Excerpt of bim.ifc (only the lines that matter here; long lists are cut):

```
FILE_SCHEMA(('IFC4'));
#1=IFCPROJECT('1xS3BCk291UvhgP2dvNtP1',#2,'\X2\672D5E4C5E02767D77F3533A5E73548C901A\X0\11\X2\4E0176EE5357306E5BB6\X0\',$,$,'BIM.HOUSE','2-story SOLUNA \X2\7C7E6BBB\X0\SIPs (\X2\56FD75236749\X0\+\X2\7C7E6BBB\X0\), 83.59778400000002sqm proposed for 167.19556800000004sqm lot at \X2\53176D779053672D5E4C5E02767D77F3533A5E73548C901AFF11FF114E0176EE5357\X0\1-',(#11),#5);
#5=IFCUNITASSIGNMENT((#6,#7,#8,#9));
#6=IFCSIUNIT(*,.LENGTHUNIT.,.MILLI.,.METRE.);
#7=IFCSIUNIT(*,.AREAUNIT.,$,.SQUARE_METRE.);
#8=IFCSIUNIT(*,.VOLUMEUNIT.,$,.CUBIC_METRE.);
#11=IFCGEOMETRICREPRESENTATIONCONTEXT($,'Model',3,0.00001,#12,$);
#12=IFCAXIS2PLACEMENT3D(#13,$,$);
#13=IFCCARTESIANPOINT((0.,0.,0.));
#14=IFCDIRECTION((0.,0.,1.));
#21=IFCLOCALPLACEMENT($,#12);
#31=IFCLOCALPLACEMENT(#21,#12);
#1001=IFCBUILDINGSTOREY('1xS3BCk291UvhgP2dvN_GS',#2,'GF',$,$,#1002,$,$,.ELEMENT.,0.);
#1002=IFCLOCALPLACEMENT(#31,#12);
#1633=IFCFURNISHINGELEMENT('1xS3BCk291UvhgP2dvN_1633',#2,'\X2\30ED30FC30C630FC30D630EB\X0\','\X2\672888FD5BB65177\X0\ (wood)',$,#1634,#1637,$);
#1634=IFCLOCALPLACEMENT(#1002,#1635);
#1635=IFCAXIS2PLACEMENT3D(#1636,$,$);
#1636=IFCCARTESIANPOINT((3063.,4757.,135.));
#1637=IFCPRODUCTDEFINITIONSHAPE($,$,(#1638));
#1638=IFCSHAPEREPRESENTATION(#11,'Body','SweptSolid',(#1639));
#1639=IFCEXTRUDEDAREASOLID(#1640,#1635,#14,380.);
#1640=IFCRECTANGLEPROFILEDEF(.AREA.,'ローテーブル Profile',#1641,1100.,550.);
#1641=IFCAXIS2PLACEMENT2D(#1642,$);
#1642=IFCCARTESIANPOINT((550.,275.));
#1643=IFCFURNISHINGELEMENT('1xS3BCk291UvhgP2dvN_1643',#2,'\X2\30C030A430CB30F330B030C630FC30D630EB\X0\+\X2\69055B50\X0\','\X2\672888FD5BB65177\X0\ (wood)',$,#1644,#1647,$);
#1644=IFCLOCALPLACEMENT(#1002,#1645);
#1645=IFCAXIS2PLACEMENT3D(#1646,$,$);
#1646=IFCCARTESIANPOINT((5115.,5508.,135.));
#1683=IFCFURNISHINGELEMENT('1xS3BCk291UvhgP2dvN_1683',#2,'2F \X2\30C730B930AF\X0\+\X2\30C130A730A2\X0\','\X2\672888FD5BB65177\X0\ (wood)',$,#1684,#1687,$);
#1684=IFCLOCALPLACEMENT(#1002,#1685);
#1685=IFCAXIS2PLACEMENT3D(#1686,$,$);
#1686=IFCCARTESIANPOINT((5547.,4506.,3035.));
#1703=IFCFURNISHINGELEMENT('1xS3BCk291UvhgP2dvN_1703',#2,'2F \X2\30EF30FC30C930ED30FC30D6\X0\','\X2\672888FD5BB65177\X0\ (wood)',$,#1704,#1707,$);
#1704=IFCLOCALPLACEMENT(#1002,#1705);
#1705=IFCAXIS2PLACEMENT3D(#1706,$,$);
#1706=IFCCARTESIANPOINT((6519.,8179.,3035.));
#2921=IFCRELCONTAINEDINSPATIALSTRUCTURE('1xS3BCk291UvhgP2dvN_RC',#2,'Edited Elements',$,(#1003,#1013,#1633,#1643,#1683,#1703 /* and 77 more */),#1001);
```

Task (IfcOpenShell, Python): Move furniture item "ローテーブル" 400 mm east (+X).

```python
import ifcopenshell
import ifcopenshell.api.geometry
import ifcopenshell.util.placement
import ifcopenshell.util.unit

model = ifcopenshell.open("bim.ifc")
unit_scale = ifcopenshell.util.unit.calculate_unit_scale(model)

item = model.by_guid("1xS3BCk291UvhgP2dvN_1633")
matrix = ifcopenshell.util.placement.get_local_placement(item.ObjectPlacement)
matrix[0, 3] += 0.4 / unit_scale
ifcopenshell.api.geometry.edit_object_placement(model, product=item, matrix=matrix, is_si=False)

print(ifcopenshell.util.placement.get_local_placement(item.ObjectPlacement).round(3) + 0.0)

model.write("bim_edited.ifc")
```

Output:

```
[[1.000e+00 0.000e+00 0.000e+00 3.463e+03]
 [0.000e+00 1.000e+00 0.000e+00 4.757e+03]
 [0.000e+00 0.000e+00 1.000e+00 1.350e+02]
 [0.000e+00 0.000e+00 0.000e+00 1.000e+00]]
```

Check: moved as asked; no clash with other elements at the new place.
